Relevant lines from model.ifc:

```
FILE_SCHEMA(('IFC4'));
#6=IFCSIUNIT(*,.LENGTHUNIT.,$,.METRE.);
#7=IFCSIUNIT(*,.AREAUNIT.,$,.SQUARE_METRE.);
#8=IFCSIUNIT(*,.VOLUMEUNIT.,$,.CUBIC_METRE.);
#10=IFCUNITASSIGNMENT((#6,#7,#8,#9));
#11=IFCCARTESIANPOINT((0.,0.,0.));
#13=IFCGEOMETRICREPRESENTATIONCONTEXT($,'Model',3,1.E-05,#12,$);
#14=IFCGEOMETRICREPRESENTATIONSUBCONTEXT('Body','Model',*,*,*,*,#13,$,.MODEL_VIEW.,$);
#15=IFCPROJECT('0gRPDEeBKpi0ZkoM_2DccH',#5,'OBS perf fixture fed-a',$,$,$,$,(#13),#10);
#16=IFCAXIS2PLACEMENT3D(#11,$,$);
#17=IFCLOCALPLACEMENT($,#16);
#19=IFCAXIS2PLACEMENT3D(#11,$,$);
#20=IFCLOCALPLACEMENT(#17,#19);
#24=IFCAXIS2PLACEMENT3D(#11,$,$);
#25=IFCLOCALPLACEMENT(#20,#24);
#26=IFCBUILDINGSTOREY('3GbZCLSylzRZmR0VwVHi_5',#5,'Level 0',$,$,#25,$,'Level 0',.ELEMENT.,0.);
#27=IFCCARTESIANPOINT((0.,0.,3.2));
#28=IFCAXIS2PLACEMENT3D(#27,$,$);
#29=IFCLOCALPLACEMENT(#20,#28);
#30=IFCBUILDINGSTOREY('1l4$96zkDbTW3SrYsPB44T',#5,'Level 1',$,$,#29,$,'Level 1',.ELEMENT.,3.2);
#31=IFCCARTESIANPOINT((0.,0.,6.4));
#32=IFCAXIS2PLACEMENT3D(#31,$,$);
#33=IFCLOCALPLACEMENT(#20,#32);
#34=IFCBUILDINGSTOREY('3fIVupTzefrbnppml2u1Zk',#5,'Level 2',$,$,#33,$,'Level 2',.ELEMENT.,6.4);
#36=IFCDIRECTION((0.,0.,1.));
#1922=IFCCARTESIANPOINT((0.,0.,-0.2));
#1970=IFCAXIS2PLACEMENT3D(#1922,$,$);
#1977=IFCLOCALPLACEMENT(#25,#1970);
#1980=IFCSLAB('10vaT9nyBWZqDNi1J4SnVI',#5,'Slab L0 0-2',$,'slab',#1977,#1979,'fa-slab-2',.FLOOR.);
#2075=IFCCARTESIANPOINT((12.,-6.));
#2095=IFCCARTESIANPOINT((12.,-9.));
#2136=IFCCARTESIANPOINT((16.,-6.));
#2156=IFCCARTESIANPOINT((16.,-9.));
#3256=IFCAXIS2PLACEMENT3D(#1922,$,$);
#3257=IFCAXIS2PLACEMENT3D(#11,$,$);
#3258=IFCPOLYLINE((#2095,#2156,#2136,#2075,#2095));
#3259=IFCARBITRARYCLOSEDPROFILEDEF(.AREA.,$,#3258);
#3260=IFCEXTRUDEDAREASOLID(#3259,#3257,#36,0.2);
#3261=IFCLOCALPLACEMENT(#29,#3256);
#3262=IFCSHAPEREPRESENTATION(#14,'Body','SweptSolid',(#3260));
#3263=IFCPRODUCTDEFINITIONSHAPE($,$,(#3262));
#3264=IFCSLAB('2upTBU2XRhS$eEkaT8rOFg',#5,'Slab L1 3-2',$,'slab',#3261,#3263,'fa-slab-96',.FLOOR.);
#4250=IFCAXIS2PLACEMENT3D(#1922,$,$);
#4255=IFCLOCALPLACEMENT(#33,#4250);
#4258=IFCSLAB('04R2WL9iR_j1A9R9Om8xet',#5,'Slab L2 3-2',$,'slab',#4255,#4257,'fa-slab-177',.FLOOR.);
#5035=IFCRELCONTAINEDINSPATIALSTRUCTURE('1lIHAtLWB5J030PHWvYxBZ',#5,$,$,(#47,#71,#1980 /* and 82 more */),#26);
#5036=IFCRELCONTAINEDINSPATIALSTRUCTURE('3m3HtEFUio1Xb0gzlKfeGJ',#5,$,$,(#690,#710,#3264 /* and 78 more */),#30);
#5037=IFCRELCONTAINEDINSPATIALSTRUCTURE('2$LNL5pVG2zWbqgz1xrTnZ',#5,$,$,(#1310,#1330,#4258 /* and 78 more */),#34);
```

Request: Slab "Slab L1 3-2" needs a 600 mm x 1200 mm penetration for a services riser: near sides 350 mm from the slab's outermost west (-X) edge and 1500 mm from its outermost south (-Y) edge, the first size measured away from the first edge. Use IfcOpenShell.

```python
import numpy as np
import ifcopenshell
import ifcopenshell.api.feature
import ifcopenshell.api.geometry
import ifcopenshell.api.root
import ifcopenshell.geom
import ifcopenshell.util.placement
import ifcopenshell.util.representation
import ifcopenshell.util.shape
import ifcopenshell.util.unit

model = ifcopenshell.open("model.ifc")
unit_scale = ifcopenshell.util.unit.calculate_unit_scale(model)
settings = ifcopenshell.geom.settings()


def volume(element):
    """Net volume in cubic metres, openings subtracted."""
    shape = ifcopenshell.geom.create_shape(settings, element)
    return ifcopenshell.util.shape.get_volume(shape.geometry)


slab = model.by_guid("2upTBU2XRhS$eEkaT8rOFg")
before = volume(slab)

# Extent in the slab's own axes, in metres. The edges named are its -X and -Y sides.
slab_shape = ifcopenshell.geom.create_shape(settings, slab)
vertices = ifcopenshell.util.shape.get_vertices(slab_shape.geometry)
x_min, y_min, bottom = vertices.min(axis=0)
top = vertices[:, 2].max()

opening = ifcopenshell.api.root.create_entity(model, ifc_class="IfcOpeningElement", name="Services riser opening", predefined_type="OPENING")
context = ifcopenshell.util.representation.get_context(model, "Model", "Body", "MODEL_VIEW")
width, depth = 0.6, 1.2
outline = [(0.0, 0.0), (width, 0.0), (width, depth), (0.0, depth), (0.0, 0.0)]
# Overshoot both faces by 50 mm so the cut is clean.
shape = ifcopenshell.api.geometry.add_slab_representation(
    model, context=context, depth=top - bottom + 0.1, polyline=outline
)
ifcopenshell.api.geometry.assign_representation(model, product=opening, representation=shape)

matrix = ifcopenshell.util.placement.get_local_placement(slab.ObjectPlacement)
matrix[:, 3] = matrix @ np.append(np.array([x_min + 0.35, y_min + 1.5, bottom - 0.05]) / unit_scale, 1.0)
ifcopenshell.api.geometry.edit_object_placement(model, product=opening, matrix=matrix, is_si=False)
ifcopenshell.api.feature.add_feature(model, feature=opening, element=slab)

after = volume(slab)

print(f"slab volume {before:.3f} -> {after:.3f} m3")

model.write("model_edited.ifc")
```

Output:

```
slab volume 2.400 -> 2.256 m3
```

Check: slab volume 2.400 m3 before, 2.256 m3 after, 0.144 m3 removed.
